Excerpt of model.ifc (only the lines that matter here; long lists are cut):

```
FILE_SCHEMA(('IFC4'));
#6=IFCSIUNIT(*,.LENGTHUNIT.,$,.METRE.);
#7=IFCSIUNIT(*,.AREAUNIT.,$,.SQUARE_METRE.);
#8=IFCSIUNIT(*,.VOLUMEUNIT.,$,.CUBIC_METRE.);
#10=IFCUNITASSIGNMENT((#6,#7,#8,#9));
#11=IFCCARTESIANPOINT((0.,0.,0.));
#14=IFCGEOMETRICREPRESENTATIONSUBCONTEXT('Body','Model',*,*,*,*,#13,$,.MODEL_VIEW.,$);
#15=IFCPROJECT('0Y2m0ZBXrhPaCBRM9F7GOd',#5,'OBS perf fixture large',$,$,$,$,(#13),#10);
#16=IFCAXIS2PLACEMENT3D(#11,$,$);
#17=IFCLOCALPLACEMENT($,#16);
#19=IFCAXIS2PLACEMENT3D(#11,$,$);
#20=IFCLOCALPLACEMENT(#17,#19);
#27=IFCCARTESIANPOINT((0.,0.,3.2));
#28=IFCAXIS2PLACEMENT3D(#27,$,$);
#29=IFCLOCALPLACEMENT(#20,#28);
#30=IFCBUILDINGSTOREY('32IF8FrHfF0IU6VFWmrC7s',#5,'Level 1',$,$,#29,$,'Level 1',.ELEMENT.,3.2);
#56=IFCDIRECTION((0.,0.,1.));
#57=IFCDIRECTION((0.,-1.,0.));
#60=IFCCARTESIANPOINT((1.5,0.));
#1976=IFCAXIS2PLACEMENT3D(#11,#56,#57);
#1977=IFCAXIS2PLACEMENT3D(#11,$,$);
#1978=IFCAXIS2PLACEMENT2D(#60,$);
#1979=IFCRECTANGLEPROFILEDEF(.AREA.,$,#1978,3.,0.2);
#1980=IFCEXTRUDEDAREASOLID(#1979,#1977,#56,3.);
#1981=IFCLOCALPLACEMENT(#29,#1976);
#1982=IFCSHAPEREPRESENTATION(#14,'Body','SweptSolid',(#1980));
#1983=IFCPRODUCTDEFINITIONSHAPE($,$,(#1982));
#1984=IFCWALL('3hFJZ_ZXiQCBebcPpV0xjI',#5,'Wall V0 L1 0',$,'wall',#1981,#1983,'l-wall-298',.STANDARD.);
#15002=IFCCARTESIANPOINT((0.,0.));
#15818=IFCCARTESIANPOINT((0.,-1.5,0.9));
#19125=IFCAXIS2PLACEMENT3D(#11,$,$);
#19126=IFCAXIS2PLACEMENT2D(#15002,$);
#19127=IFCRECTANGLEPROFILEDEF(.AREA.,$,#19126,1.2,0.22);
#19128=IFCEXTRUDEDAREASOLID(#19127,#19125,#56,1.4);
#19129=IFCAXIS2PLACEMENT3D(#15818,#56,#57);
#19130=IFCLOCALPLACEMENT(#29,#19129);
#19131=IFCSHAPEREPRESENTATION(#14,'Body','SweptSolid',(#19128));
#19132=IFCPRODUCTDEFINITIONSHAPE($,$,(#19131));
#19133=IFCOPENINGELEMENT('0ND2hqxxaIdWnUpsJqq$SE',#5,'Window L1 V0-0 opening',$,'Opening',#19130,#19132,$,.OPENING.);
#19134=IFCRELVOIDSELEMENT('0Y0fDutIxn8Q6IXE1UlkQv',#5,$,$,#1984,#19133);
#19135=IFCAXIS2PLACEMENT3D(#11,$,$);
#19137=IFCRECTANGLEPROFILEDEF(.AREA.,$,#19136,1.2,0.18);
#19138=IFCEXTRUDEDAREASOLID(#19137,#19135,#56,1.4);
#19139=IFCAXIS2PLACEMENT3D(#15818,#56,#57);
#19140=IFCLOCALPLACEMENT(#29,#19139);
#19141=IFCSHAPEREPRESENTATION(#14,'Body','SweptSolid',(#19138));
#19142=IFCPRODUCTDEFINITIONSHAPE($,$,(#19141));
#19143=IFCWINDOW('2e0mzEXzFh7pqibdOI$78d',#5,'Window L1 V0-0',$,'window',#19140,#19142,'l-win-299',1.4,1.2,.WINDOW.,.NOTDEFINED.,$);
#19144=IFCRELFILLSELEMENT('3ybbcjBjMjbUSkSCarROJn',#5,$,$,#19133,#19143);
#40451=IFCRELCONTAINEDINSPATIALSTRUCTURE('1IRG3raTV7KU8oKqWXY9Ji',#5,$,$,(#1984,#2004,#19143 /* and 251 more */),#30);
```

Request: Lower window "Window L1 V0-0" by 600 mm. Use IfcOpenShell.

```python
import numpy as np
import ifcopenshell
import ifcopenshell.api.geometry
import ifcopenshell.util.placement
import ifcopenshell.util.unit

model = ifcopenshell.open("model.ifc")
unit_scale = ifcopenshell.util.unit.calculate_unit_scale(model)

window = model.by_guid("2e0mzEXzFh7pqibdOI$78d")
opening = window.FillsVoids[0].RelatingOpeningElement
dz = -0.6 / unit_scale

shift = np.array([0.0, 0.0, dz])
# The window is not placed relative to its opening, so move both.
for product in (opening, window):
    matrix = ifcopenshell.util.placement.get_local_placement(product.ObjectPlacement)
    matrix[:3, 3] += shift
    ifcopenshell.api.geometry.edit_object_placement(model, product=product, matrix=matrix, is_si=False)

print(f"moved by {dz * unit_scale:+.3f} m")

model.write("model_updated.ifc")
```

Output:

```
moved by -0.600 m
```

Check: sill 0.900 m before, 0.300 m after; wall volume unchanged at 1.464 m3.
